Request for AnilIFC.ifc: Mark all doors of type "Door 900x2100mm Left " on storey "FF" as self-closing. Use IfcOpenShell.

First a look at what the model holds.

```python
import ifcopenshell
import ifcopenshell.util.element

model = ifcopenshell.open("AnilIFC.ifc")
print(model.schema)
storey = next(s for s in model.by_type("IfcBuildingStorey") if s.Name == "FF")
doors = [e for e in ifcopenshell.util.element.get_decomposition(storey) if e.is_a("IfcDoor")]
seen = {}
for e in doors:
    element_type = ifcopenshell.util.element.get_type(e)
    key = (element_type.Name if element_type != e and element_type else None, ifcopenshell.util.element.get_pset(e, "Pset_DoorCommon", "SelfClosing"))
    seen[key] = seen.get(key, 0) + 1
for (name, value), count in sorted(seen.items(), key=str):
    print(count, "x", name, "|", value)
```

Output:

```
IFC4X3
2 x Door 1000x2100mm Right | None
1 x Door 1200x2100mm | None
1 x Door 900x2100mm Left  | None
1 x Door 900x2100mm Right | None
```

```python
import ifcopenshell
import ifcopenshell.api.pset
import ifcopenshell.util.element

model = ifcopenshell.open("AnilIFC.ifc")

storey = next(s for s in model.by_type("IfcBuildingStorey") if s.Name == "FF")
doors = [e for e in ifcopenshell.util.element.get_decomposition(storey) if e.is_a("IfcDoor")]

count = 0
for e in doors:
    element_type = ifcopenshell.util.element.get_type(e)
    if element_type in (None, e) or element_type.Name != "Door 900x2100mm Left ":
        continue
    # add_pset returns the element's existing set when there is one.
    pset = ifcopenshell.api.pset.add_pset(model, product=e, name="Pset_DoorCommon")
    ifcopenshell.api.pset.edit_pset(model, pset=pset, properties={"SelfClosing": True})
    count += 1

print(count, "doors updated")

model.write("AnilIFC_edited.ifc")
```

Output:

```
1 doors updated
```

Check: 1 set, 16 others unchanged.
